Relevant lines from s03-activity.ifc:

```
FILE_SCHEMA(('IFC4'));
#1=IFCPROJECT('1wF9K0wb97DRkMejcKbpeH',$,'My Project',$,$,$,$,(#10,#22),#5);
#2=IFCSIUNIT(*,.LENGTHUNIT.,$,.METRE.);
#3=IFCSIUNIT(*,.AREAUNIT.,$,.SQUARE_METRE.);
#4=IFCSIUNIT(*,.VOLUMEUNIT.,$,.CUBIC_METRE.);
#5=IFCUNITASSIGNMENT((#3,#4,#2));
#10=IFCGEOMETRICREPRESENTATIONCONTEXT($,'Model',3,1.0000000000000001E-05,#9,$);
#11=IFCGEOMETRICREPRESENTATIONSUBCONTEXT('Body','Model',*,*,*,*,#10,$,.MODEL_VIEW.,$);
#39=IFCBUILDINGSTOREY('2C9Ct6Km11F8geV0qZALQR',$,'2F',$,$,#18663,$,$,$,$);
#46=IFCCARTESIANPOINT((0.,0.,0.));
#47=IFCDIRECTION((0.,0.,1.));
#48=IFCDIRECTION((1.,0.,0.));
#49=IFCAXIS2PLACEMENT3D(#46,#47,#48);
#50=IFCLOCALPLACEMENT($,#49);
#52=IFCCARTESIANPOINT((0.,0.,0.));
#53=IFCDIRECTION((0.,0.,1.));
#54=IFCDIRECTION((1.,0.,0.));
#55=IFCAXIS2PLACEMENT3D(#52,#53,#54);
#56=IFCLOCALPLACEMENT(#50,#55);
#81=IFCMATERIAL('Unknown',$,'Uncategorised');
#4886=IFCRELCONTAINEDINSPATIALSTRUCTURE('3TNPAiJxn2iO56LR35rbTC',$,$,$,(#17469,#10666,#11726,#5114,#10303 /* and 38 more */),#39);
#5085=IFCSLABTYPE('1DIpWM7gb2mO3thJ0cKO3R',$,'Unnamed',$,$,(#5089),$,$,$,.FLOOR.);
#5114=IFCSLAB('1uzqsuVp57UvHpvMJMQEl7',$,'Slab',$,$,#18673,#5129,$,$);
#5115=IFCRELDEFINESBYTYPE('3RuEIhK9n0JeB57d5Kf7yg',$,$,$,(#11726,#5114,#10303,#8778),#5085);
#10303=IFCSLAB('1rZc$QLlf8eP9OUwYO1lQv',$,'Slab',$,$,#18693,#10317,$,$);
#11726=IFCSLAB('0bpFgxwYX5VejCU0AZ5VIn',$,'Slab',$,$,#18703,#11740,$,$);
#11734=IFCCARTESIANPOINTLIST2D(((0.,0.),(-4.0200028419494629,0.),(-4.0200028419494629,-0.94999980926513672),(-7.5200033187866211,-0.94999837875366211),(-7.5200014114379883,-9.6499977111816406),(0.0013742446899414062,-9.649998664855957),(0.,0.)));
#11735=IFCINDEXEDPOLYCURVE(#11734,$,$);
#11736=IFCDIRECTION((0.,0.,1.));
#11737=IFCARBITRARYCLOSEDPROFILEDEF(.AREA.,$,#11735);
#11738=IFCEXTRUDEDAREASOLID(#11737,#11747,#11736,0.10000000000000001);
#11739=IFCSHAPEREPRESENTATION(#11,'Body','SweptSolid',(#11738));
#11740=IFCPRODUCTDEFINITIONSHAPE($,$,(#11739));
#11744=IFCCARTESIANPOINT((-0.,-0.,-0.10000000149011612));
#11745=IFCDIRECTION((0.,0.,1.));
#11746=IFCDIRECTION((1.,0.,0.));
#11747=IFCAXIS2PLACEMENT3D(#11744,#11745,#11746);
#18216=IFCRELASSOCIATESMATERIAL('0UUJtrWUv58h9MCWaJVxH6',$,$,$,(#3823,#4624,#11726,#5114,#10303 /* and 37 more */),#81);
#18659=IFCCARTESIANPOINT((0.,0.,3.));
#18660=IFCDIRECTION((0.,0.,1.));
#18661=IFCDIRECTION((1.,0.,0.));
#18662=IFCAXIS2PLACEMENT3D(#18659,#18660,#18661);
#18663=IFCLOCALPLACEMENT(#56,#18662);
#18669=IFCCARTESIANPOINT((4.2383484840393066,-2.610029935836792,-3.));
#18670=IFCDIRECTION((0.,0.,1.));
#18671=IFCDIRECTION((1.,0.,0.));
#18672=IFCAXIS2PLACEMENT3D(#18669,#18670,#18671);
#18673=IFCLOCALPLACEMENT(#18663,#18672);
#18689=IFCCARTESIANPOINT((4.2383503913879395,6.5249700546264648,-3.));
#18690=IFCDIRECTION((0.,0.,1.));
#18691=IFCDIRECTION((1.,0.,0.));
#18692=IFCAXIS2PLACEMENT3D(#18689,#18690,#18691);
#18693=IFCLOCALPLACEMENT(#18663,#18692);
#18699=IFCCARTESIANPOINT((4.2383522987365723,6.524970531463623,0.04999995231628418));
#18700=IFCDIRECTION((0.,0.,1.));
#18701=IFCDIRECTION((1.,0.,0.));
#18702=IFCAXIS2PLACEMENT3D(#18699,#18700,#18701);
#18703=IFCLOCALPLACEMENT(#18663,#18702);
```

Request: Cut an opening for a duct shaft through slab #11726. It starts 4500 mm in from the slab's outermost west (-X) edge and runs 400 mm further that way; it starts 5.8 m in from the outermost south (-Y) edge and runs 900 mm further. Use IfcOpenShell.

```python
import numpy as np
import ifcopenshell
import ifcopenshell.api.feature
import ifcopenshell.api.geometry
import ifcopenshell.api.root
import ifcopenshell.geom
import ifcopenshell.util.placement
import ifcopenshell.util.representation
import ifcopenshell.util.shape
import ifcopenshell.util.unit

model = ifcopenshell.open("s03-activity.ifc")
unit_scale = ifcopenshell.util.unit.calculate_unit_scale(model)
settings = ifcopenshell.geom.settings()


def volume(element):
    """Net volume in cubic metres, openings subtracted."""
    shape = ifcopenshell.geom.create_shape(settings, element)
    return ifcopenshell.util.shape.get_volume(shape.geometry)


slab = model.by_guid("0bpFgxwYX5VejCU0AZ5VIn")
before = volume(slab)

# Extent in the slab's own axes, in metres. The edges named are its -X and -Y sides.
slab_shape = ifcopenshell.geom.create_shape(settings, slab)
vertices = ifcopenshell.util.shape.get_vertices(slab_shape.geometry)
x_min, y_min, bottom = vertices.min(axis=0)
top = vertices[:, 2].max()

opening = ifcopenshell.api.root.create_entity(model, ifc_class="IfcOpeningElement", name="Duct shaft opening", predefined_type="OPENING")
context = ifcopenshell.util.representation.get_context(model, "Model", "Body", "MODEL_VIEW")
width, depth = 0.4, 0.9
outline = [(0.0, 0.0), (width, 0.0), (width, depth), (0.0, depth), (0.0, 0.0)]
# Overshoot both faces by 50 mm so the cut is clean.
shape = ifcopenshell.api.geometry.add_slab_representation(
    model, context=context, depth=top - bottom + 0.1, polyline=outline
)
ifcopenshell.api.geometry.assign_representation(model, product=opening, representation=shape)

matrix = ifcopenshell.util.placement.get_local_placement(slab.ObjectPlacement)
matrix[:, 3] = matrix @ np.append(np.array([x_min + 4.5, y_min + 5.8, bottom - 0.05]) / unit_scale, 1.0)
ifcopenshell.api.geometry.edit_object_placement(model, product=opening, matrix=matrix, is_si=False)
ifcopenshell.api.feature.add_feature(model, feature=opening, element=slab)

after = volume(slab)

print(f"slab volume {before:.3f} -> {after:.3f} m3")

model.write("s03-activity-out.ifc")
```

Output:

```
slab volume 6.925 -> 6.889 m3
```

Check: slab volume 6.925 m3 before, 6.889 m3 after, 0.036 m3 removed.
